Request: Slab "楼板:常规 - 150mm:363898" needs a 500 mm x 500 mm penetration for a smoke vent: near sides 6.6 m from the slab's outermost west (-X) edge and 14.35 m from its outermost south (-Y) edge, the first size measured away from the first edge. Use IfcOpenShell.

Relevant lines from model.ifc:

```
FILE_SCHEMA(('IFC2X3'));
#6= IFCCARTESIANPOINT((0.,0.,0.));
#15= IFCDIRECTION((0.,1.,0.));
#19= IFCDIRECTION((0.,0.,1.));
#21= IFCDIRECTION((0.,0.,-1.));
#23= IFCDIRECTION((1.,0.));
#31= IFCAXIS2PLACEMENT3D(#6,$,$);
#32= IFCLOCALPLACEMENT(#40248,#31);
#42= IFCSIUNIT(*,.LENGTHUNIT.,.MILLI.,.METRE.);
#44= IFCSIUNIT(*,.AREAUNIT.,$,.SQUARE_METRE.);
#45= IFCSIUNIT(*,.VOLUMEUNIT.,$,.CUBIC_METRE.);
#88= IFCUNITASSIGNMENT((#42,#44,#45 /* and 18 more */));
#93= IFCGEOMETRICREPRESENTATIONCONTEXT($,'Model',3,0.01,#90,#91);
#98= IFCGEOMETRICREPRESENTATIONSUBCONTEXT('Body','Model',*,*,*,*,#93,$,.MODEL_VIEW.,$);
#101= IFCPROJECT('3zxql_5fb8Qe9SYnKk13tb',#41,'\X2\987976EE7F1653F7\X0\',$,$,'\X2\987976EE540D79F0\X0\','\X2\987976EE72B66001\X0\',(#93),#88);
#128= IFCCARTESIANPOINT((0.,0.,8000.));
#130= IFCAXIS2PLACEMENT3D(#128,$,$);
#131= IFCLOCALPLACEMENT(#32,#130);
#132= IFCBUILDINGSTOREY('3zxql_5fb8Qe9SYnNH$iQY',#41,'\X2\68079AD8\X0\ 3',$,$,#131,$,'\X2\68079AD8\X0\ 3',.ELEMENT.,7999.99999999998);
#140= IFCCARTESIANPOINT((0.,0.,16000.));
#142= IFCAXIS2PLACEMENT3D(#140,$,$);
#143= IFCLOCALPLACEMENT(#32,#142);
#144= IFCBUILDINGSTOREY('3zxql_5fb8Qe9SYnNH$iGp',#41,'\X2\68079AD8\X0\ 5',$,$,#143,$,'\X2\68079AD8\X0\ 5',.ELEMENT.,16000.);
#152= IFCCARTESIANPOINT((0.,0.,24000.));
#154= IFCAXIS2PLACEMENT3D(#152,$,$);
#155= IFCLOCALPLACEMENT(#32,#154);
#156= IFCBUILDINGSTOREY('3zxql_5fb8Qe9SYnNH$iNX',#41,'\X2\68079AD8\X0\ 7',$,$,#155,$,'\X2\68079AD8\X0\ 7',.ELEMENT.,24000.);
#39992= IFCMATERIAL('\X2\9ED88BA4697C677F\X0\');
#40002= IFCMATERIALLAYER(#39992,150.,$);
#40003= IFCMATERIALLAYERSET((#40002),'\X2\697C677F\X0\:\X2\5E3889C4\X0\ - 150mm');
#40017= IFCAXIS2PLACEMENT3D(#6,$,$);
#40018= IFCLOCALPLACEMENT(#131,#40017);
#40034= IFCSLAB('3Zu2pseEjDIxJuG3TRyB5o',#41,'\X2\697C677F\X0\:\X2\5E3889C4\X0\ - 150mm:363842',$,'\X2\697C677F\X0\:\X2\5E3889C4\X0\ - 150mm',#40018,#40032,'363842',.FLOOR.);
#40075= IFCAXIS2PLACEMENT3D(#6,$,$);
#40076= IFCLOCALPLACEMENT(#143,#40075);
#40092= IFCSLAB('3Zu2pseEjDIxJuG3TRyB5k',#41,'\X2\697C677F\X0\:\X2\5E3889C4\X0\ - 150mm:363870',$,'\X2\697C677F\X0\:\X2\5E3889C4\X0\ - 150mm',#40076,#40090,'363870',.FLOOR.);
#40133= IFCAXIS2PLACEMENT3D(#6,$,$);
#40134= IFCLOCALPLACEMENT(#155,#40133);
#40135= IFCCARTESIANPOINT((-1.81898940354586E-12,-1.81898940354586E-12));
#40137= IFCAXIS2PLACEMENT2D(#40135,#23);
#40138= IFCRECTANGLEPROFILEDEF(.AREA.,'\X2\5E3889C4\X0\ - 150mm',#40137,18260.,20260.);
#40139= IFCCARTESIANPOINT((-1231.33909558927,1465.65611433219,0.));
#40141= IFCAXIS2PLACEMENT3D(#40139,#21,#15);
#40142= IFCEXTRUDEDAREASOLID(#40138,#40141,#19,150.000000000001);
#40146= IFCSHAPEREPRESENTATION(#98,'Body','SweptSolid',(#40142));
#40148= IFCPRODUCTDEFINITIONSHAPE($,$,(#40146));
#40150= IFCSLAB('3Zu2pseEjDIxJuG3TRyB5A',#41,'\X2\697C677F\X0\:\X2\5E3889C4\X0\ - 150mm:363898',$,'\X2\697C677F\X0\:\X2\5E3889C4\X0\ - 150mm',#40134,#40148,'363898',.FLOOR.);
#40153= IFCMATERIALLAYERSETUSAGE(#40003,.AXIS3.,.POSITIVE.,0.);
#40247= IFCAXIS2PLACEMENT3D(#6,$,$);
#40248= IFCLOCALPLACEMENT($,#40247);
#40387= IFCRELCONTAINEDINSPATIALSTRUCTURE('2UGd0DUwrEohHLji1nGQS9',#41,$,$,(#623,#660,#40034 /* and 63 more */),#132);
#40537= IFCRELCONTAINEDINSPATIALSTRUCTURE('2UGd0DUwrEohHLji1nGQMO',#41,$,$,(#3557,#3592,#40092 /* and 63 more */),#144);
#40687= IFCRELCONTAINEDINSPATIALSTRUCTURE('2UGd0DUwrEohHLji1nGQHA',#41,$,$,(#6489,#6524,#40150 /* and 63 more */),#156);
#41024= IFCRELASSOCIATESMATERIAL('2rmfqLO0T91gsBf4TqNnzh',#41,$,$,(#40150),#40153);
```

```python
import numpy as np
import ifcopenshell
import ifcopenshell.api.feature
import ifcopenshell.api.geometry
import ifcopenshell.api.root
import ifcopenshell.geom
import ifcopenshell.util.placement
import ifcopenshell.util.representation
import ifcopenshell.util.shape
import ifcopenshell.util.unit

model = ifcopenshell.open("model.ifc")
unit_scale = ifcopenshell.util.unit.calculate_unit_scale(model)
settings = ifcopenshell.geom.settings()


def volume(element):
    """Net volume in cubic metres, openings subtracted."""
    shape = ifcopenshell.geom.create_shape(settings, element)
    return ifcopenshell.util.shape.get_volume(shape.geometry)


slab = model.by_id(40150)
before = volume(slab)

# Extent in the slab's own axes, in metres. The edges named are its -X and -Y sides.
slab_shape = ifcopenshell.geom.create_shape(settings, slab)
vertices = ifcopenshell.util.shape.get_vertices(slab_shape.geometry)
x_min, y_min, bottom = vertices.min(axis=0)
top = vertices[:, 2].max()

opening = ifcopenshell.api.root.create_entity(model, ifc_class="IfcOpeningElement", name="Smoke vent opening")
context = ifcopenshell.util.representation.get_context(model, "Model", "Body", "MODEL_VIEW")
width, depth = 0.5, 0.5
outline = [(0.0, 0.0), (width, 0.0), (width, depth), (0.0, depth), (0.0, 0.0)]
# Overshoot both faces by 50 mm so the cut is clean.
shape = ifcopenshell.api.geometry.add_slab_representation(
    model, context=context, depth=top - bottom + 0.1, polyline=outline
)
ifcopenshell.api.geometry.assign_representation(model, product=opening, representation=shape)

matrix = ifcopenshell.util.placement.get_local_placement(slab.ObjectPlacement)
matrix[:, 3] = matrix @ np.append(np.array([x_min + 6.6, y_min + 14.35, bottom - 0.05]) / unit_scale, 1.0)
ifcopenshell.api.geometry.edit_object_placement(model, product=opening, matrix=matrix, is_si=False)
ifcopenshell.api.feature.add_feature(model, feature=opening, element=slab)

after = volume(slab)

print(f"slab volume {before:.3f} -> {after:.3f} m3")

model.write("model_edited.ifc")
```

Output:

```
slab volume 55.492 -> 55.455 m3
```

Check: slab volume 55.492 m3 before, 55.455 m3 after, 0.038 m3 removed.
